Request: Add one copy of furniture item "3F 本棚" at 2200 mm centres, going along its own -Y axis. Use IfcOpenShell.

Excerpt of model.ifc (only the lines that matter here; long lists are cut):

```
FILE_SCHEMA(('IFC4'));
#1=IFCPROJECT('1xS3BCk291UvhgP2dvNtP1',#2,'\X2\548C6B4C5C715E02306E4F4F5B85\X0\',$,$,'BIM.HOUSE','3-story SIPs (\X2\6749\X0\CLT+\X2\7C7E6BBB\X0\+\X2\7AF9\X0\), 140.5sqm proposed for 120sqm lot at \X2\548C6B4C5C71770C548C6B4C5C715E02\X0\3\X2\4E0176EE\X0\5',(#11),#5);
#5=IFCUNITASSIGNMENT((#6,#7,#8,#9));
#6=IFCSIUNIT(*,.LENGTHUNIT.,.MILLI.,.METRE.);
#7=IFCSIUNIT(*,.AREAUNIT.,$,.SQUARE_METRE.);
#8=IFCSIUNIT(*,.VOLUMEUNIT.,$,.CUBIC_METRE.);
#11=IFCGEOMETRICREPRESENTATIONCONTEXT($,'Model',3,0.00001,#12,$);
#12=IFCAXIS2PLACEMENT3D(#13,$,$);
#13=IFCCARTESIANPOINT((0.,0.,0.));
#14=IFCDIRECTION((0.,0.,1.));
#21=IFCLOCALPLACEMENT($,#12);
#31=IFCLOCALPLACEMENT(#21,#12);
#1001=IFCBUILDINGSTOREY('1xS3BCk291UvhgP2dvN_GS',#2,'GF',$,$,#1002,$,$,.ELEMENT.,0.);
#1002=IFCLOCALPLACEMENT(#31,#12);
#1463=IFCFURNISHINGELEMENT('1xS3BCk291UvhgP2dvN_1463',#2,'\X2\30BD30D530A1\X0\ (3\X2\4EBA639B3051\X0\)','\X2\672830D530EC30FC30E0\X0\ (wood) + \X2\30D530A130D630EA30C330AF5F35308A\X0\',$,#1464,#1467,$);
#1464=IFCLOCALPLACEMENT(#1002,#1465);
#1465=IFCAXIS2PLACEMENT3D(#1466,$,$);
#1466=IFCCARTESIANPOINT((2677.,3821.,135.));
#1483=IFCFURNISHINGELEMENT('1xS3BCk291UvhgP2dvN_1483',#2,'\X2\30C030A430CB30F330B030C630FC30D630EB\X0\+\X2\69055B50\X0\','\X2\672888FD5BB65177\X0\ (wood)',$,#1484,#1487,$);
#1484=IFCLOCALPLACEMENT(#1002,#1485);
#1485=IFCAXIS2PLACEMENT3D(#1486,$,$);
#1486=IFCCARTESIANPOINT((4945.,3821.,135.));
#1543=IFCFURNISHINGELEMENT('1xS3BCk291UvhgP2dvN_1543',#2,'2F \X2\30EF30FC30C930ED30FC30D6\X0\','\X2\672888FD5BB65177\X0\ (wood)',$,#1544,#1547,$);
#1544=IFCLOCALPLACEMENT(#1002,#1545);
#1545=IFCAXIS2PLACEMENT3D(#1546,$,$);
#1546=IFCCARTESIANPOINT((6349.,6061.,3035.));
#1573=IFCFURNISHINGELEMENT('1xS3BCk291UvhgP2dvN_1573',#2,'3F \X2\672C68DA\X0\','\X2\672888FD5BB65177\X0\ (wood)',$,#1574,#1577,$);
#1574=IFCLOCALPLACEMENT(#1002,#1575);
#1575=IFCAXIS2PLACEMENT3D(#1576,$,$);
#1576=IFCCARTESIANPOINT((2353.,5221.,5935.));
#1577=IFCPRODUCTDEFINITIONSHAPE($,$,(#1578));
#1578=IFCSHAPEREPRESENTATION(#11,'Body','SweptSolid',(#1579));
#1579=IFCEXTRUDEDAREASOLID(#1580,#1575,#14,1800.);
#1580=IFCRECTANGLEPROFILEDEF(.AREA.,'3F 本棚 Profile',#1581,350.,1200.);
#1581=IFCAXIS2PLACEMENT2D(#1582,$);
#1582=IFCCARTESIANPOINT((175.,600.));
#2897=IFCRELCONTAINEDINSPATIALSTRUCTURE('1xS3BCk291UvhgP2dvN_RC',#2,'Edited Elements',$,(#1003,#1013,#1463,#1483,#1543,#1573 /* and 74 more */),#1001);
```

```python
import ifcopenshell
import ifcopenshell.api.geometry
import ifcopenshell.api.root
import ifcopenshell.util.element
import ifcopenshell.util.placement

model = ifcopenshell.open("model.ifc")


def reuse_history(source, copy):
    """copy_class also copies each property set's owner history, people and application; keep the originals."""
    for rel in copy.IsDefinedBy:
        if rel.is_a("IfcRelDefinesByProperties") and (history := rel.RelatingPropertyDefinition.OwnerHistory):
            rel.RelatingPropertyDefinition.OwnerHistory = source.OwnerHistory
            ifcopenshell.util.element.remove_deep2(model, history)


source = model.by_id(1573)
base = ifcopenshell.util.placement.get_local_placement(source.ObjectPlacement)
step = -base[:3, 1] * 2200.0

for i in range(1, 2):
    copy = ifcopenshell.api.root.copy_class(model, product=source)
    copy.Representation = ifcopenshell.util.element.copy_deep(
        model, source.Representation, exclude=["IfcGeometricRepresentationContext", "IfcRepresentationMap"]
    )
    reuse_history(source, copy)
    matrix = base.copy()
    matrix[:3, 3] += i * step
    print("added at", matrix[:3, 3].round(3) + 0.0)
    ifcopenshell.api.geometry.edit_object_placement(model, product=copy, matrix=matrix, is_si=False)

model.write("model_v2.ifc")
```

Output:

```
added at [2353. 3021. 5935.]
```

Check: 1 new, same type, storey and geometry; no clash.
